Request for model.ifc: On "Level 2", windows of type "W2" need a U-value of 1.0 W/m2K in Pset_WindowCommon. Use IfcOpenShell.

First a look at what the model holds.

```python
import ifcopenshell
import ifcopenshell.util.element

model = ifcopenshell.open("model.ifc")
print(model.schema)
storey = next(s for s in model.by_type("IfcBuildingStorey") if s.Name == "Level 2")
windows = [e for e in ifcopenshell.util.element.get_decomposition(storey) if e.is_a("IfcWindow")]
seen = {}
for e in windows:
    element_type = ifcopenshell.util.element.get_type(e)
    key = (element_type.Name if element_type != e and element_type else None, ifcopenshell.util.element.get_pset(e, "Pset_WindowCommon", "ThermalTransmittance"))
    seen[key] = seen.get(key, 0) + 1
for (name, value), count in sorted(seen.items(), key=str):
    print(count, "x", name, "|", value)
```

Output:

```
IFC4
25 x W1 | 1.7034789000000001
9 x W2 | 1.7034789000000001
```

```python
import ifcopenshell
import ifcopenshell.api.pset
import ifcopenshell.util.element

model = ifcopenshell.open("model.ifc")

storey = next(s for s in model.by_type("IfcBuildingStorey") if s.Name == "Level 2")
windows = [e for e in ifcopenshell.util.element.get_decomposition(storey) if e.is_a("IfcWindow")]

count = 0
for e in windows:
    element_type = ifcopenshell.util.element.get_type(e)
    if element_type in (None, e) or element_type.Name != "W2":
        continue
    # add_pset returns the element's existing set when there is one.
    pset = ifcopenshell.api.pset.add_pset(model, product=e, name="Pset_WindowCommon")
    ifcopenshell.api.pset.edit_pset(model, pset=pset, properties={"ThermalTransmittance": 1.0})
    count += 1

print(count, "windows updated")

model.write("model_edited.ifc")
```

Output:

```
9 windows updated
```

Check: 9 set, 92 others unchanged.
